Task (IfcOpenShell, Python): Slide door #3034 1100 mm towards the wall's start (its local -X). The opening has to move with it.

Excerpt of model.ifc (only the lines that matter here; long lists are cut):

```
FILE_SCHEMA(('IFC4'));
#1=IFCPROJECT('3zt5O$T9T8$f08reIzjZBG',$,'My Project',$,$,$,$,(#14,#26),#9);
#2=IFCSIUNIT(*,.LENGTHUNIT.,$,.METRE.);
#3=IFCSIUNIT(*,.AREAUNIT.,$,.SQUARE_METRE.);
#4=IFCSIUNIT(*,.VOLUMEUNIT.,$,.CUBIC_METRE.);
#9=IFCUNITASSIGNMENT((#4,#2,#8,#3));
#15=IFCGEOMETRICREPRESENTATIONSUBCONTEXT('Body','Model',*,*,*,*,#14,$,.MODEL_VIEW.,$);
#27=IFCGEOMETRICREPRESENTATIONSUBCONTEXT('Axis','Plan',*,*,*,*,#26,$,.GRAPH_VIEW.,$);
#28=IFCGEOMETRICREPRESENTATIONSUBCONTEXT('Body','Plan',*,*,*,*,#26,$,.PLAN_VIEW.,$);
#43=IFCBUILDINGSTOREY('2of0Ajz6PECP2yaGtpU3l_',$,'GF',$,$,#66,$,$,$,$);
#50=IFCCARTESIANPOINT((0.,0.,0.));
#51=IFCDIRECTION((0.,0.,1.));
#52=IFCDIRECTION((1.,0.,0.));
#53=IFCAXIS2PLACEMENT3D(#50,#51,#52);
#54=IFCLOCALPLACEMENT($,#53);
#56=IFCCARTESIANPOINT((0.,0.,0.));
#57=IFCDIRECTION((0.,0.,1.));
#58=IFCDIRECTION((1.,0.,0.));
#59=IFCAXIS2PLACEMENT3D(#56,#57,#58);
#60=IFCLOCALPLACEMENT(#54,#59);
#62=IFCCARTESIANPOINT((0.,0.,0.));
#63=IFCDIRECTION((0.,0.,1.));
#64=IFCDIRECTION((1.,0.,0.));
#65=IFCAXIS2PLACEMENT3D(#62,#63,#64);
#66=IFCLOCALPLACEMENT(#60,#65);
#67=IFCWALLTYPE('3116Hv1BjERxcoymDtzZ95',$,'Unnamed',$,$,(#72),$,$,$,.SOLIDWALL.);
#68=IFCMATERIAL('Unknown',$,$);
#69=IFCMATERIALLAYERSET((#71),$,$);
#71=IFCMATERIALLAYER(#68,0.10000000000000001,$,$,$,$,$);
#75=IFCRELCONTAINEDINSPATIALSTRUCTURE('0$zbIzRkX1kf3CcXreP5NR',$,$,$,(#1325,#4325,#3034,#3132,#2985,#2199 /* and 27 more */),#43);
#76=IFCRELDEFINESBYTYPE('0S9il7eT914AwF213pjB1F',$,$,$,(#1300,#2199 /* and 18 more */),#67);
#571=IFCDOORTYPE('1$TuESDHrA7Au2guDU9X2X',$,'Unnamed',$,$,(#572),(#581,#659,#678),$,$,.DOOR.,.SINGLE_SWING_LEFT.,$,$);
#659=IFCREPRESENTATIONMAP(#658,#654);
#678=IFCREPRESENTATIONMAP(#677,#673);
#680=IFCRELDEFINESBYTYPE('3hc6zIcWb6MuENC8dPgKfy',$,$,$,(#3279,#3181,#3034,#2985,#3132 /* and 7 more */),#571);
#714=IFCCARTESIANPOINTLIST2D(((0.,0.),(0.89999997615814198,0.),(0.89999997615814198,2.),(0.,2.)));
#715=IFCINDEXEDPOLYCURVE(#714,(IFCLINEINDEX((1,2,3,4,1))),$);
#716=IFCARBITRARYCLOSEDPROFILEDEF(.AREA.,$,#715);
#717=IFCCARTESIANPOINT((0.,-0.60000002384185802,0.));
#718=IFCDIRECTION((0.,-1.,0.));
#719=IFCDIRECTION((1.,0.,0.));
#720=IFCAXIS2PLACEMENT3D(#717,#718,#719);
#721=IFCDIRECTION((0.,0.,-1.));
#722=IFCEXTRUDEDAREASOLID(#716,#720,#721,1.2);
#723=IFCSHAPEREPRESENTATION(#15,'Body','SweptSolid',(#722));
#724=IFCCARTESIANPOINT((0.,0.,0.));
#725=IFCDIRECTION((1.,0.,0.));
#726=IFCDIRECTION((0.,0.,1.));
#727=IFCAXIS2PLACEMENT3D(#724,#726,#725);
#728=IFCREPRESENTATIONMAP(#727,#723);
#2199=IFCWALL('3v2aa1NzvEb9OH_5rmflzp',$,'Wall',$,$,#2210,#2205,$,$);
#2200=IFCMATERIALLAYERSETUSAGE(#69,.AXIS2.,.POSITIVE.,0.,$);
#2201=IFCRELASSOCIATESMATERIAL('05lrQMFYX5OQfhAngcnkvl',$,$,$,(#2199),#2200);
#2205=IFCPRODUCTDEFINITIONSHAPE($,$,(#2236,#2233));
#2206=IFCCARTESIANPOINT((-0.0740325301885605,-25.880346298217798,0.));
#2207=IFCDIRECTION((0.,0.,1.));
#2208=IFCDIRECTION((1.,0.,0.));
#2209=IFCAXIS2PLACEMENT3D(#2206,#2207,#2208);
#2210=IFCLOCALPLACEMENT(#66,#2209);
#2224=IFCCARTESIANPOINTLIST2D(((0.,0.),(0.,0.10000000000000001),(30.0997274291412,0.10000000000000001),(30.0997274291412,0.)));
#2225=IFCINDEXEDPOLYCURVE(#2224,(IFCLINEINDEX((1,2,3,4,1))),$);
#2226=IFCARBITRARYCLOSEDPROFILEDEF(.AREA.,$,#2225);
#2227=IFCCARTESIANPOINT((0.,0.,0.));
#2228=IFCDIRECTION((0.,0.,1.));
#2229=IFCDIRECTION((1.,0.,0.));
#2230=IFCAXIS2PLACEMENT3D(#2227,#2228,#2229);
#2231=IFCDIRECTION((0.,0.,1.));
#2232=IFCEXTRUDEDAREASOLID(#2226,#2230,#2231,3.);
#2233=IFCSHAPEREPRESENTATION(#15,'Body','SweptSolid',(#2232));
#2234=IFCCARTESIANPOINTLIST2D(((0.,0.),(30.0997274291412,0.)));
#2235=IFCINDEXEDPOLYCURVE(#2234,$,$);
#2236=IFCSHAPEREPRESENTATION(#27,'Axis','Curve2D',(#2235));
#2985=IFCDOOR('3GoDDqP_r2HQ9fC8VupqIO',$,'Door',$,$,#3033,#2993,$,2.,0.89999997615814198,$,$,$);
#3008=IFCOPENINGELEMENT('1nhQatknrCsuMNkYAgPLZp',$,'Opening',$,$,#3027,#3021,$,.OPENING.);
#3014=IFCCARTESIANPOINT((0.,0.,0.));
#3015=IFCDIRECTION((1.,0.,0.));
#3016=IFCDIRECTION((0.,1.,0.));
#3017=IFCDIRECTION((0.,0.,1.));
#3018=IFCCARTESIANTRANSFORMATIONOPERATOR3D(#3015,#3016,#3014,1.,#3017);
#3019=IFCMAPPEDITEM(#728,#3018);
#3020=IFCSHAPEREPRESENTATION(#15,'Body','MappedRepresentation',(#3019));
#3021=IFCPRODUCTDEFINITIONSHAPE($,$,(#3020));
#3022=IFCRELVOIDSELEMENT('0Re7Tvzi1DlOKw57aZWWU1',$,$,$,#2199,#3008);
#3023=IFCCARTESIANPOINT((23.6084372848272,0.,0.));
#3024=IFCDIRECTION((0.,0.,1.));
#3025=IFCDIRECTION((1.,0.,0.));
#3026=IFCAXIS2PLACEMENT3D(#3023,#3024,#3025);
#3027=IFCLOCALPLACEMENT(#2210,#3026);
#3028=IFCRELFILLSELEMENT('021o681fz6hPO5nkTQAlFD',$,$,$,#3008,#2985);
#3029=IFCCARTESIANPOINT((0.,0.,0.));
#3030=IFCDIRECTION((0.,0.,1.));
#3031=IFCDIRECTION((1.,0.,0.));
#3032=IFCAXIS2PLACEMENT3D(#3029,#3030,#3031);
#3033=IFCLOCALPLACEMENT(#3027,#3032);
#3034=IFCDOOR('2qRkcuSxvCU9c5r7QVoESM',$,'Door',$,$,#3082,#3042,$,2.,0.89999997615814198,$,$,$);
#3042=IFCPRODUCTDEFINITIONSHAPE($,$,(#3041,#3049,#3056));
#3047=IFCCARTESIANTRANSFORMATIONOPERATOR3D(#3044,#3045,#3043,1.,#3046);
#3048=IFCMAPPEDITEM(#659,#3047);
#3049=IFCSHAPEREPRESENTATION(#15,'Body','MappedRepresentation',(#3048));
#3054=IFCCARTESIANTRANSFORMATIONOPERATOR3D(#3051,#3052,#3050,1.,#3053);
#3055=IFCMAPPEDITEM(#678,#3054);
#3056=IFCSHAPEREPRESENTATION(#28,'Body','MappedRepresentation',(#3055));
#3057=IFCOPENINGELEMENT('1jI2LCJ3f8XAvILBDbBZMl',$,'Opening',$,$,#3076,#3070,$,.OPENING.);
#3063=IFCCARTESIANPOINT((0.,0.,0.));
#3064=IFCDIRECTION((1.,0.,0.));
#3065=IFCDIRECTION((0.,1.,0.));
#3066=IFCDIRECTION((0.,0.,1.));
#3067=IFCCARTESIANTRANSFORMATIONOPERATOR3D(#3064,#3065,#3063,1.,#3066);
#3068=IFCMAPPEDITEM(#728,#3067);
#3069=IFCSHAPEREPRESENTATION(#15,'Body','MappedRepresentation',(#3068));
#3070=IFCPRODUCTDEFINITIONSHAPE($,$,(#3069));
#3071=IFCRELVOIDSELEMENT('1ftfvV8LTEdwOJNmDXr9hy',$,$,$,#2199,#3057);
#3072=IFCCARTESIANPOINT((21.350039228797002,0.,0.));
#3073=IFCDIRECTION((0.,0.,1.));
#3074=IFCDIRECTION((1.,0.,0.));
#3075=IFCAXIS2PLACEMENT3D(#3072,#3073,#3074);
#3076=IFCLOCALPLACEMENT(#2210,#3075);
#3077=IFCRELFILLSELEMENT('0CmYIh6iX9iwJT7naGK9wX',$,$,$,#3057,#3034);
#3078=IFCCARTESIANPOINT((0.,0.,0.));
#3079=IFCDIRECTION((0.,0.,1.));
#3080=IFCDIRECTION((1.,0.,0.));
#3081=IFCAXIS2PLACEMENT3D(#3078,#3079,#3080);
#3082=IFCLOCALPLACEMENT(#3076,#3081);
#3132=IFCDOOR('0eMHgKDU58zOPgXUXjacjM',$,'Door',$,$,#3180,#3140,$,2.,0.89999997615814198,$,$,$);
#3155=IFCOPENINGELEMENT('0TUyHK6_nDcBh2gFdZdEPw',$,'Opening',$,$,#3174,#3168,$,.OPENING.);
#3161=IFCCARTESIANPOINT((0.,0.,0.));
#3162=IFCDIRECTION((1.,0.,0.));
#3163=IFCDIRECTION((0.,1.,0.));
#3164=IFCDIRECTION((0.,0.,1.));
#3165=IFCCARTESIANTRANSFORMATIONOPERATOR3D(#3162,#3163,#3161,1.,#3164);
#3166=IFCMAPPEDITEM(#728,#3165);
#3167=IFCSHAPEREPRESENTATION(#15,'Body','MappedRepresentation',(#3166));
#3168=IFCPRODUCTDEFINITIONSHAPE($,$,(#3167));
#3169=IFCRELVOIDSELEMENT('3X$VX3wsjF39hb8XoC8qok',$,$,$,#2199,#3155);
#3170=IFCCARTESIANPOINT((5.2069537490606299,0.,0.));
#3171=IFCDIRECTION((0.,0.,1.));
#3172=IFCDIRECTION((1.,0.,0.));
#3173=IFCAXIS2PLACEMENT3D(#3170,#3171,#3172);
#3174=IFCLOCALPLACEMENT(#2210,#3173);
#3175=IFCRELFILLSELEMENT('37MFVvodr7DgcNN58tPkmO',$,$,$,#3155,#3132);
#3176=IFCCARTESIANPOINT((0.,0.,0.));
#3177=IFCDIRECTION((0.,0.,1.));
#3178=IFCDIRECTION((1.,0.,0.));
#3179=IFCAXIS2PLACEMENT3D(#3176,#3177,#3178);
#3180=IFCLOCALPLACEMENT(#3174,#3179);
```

```python
import ifcopenshell
import ifcopenshell.api.geometry
import ifcopenshell.util.placement

model = ifcopenshell.open("model.ifc")

door = model.by_guid("2qRkcuSxvCU9c5r7QVoESM")
opening = door.FillsVoids[0].RelatingOpeningElement
wall = opening.VoidsElements[0].RelatingBuildingElement

wall_matrix = ifcopenshell.util.placement.get_local_placement(wall.ObjectPlacement)
shift = wall_matrix[:3, 0] * -1.1
before = ifcopenshell.util.placement.get_local_placement(door.ObjectPlacement)[:3, 3].copy()

# The door is placed relative to its opening, so it follows when the opening moves.
matrix = ifcopenshell.util.placement.get_local_placement(opening.ObjectPlacement)
matrix[:3, 3] += shift
ifcopenshell.api.geometry.edit_object_placement(
    model, product=opening, matrix=matrix, is_si=False, should_transform_children=True
)

after = ifcopenshell.util.placement.get_local_placement(door.ObjectPlacement)[:3, 3]
print("door moved by", (after - before).round(3) + 0.0)

model.write("model_edited.ifc")
```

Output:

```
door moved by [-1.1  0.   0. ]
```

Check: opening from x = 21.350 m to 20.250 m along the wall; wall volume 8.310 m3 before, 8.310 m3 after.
